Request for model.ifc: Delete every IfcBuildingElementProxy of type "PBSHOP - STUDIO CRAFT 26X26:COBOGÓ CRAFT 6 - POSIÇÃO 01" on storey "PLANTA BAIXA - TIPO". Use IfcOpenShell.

First a look at what the model holds.

```python
import ifcopenshell
import ifcopenshell.util.element

model = ifcopenshell.open("model.ifc")
print(model.schema)
storey = next(s for s in model.by_type("IfcBuildingStorey") if s.Name == "PLANTA BAIXA - TIPO")
proxies = [e for e in ifcopenshell.util.element.get_decomposition(storey) if e.is_a("IfcBuildingElementProxy")]
seen = {}
for e in proxies:
    element_type = ifcopenshell.util.element.get_type(e)
    name = element_type.Name if element_type not in (None, e) else None
    seen[name] = seen.get(name, 0) + 1
for name, count in sorted(seen.items(), key=str):
    print(count, "x", name)
```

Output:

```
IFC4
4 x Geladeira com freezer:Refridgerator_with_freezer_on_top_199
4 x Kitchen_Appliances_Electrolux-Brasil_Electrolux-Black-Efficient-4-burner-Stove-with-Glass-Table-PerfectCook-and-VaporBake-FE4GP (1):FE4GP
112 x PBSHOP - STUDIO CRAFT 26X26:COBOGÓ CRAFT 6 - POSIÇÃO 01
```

```python
import ifcopenshell
import ifcopenshell.api.root
import ifcopenshell.util.element

model = ifcopenshell.open("model.ifc")

storey = next(s for s in model.by_type("IfcBuildingStorey") if s.Name == "PLANTA BAIXA - TIPO")
proxies = [e for e in ifcopenshell.util.element.get_decomposition(storey) if e.is_a("IfcBuildingElementProxy")]
targets = [e for e in proxies if (t := ifcopenshell.util.element.get_type(e)) not in (None, e) and t.Name == "PBSHOP - STUDIO CRAFT 26X26:COBOGÓ CRAFT 6 - POSIÇÃO 01"]

for e in targets:
    ifcopenshell.api.root.remove_product(model, product=e)
print(len(targets), "removed")

model.write("model-out.ifc")
```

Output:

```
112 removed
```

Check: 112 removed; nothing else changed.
